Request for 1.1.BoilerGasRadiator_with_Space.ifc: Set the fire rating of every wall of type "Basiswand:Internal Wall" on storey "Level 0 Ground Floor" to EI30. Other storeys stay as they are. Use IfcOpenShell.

First a look at what the model holds.

```python
import ifcopenshell
import ifcopenshell.util.element

model = ifcopenshell.open("1.1.BoilerGasRadiator_with_Space.ifc")
print(model.schema)
storey = next(s for s in model.by_type("IfcBuildingStorey") if s.Name == "Level 0 Ground Floor")
walls = [e for e in ifcopenshell.util.element.get_decomposition(storey) if e.is_a("IfcWall")]
seen = {}
for e in walls:
    element_type = ifcopenshell.util.element.get_type(e)
    key = (element_type.Name if element_type != e and element_type else None, ifcopenshell.util.element.get_pset(e, "Pset_WallCommon", "FireRating"))
    seen[key] = seen.get(key, 0) + 1
for (name, value), count in sorted(seen.items(), key=str):
    print(count, "x", name, "|", value)
```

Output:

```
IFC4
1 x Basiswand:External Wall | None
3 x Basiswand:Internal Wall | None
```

```python
import ifcopenshell
import ifcopenshell.api.pset
import ifcopenshell.util.element

model = ifcopenshell.open("1.1.BoilerGasRadiator_with_Space.ifc")

storey = next(s for s in model.by_type("IfcBuildingStorey") if s.Name == "Level 0 Ground Floor")
walls = [e for e in ifcopenshell.util.element.get_decomposition(storey) if e.is_a("IfcWall")]

count = 0
for e in walls:
    element_type = ifcopenshell.util.element.get_type(e)
    if element_type in (None, e) or element_type.Name != "Basiswand:Internal Wall":
        continue
    # add_pset returns the element's existing set when there is one.
    pset = ifcopenshell.api.pset.add_pset(model, product=e, name="Pset_WallCommon")
    ifcopenshell.api.pset.edit_pset(model, pset=pset, properties={"FireRating": "EI30"})
    count += 1

print(count, "walls updated")

model.write("1.1.BoilerGasRadiator_with_Space-out.ifc")
```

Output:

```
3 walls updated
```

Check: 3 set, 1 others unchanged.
